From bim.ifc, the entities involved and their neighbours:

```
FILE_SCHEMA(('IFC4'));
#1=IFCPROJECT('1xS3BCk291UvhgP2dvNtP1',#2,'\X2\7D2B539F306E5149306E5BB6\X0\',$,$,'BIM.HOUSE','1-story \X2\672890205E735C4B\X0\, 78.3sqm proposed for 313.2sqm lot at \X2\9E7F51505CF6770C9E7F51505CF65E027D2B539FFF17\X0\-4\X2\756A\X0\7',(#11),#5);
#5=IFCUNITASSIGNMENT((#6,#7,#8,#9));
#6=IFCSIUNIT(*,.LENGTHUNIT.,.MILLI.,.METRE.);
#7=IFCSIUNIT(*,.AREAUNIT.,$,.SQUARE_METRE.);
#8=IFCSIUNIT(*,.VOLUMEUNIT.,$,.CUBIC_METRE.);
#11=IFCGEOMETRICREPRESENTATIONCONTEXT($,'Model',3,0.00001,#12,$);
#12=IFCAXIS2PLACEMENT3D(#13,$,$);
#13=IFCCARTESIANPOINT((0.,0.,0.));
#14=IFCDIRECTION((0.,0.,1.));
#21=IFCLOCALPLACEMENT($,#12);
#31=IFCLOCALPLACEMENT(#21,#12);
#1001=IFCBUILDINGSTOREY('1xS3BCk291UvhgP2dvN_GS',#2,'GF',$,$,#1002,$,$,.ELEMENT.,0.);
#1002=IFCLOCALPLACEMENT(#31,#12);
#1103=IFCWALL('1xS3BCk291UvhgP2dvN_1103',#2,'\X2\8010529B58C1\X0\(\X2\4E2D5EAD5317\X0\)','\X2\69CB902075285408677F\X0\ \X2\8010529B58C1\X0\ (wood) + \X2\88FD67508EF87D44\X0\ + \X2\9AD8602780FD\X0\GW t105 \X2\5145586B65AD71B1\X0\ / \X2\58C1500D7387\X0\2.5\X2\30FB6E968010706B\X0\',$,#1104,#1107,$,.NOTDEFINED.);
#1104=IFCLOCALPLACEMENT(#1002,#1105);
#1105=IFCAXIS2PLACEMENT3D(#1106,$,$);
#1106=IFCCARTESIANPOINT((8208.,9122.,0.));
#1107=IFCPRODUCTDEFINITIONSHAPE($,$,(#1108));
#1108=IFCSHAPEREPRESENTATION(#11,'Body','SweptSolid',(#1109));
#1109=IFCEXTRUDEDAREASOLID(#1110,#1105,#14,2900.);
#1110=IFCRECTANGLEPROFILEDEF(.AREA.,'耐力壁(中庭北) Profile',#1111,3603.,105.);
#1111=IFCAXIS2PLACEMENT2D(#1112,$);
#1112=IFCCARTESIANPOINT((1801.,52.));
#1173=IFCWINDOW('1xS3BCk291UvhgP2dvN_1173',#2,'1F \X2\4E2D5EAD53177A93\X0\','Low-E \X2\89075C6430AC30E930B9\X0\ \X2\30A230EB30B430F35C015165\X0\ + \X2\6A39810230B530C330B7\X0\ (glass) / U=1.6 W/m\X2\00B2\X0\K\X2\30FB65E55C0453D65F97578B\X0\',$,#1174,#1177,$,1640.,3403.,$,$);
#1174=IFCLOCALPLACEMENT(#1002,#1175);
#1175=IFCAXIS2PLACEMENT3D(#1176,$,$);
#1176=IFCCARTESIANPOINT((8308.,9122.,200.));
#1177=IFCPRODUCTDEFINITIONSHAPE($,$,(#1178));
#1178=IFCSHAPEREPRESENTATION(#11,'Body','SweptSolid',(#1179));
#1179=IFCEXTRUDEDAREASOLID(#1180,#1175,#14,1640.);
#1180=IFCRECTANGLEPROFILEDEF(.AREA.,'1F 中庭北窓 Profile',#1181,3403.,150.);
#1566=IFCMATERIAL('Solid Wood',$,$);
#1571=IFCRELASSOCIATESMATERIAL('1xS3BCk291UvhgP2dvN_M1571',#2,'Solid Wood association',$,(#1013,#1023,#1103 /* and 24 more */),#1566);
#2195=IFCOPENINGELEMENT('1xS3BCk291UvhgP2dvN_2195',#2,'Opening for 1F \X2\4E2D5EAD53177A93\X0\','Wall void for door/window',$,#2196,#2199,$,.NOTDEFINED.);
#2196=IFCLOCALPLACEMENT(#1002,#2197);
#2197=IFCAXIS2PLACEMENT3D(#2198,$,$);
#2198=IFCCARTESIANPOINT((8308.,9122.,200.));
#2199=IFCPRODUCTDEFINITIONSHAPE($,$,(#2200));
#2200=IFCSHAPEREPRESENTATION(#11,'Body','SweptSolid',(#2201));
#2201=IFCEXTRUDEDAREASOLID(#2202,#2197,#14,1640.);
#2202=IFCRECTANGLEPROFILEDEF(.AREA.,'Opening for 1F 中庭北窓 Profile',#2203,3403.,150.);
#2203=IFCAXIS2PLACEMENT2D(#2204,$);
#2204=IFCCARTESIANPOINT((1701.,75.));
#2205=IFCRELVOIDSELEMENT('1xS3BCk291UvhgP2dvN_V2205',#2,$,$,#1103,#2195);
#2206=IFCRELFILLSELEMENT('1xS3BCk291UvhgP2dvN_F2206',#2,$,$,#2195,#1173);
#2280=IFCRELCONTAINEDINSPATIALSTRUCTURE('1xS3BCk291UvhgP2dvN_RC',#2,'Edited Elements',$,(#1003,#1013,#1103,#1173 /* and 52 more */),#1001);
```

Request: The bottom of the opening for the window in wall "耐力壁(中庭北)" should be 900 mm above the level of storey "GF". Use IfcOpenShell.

```python
import numpy as np
import ifcopenshell
import ifcopenshell.api.geometry
import ifcopenshell.geom
import ifcopenshell.util.element
import ifcopenshell.util.placement
import ifcopenshell.util.shape
import ifcopenshell.util.unit

model = ifcopenshell.open("bim.ifc")
unit_scale = ifcopenshell.util.unit.calculate_unit_scale(model)

window = model.by_id(1173)
opening = window.FillsVoids[0].RelatingOpeningElement
storey = ifcopenshell.util.element.get_container(window, ifc_class="IfcBuildingStorey")
level = ifcopenshell.util.placement.get_local_placement(storey.ObjectPlacement)[2, 3]

# The opening's origin need not be at the sill, so measure its lowest point.
shape = ifcopenshell.geom.create_shape(ifcopenshell.geom.settings(), opening)
bottom = ifcopenshell.util.shape.get_shape_bottom_elevation(shape, shape.geometry) / unit_scale
dz = level + 0.9 / unit_scale - bottom

shift = np.array([0.0, 0.0, dz])
# The window is not placed relative to its opening, so move both.
for product in (opening, window):
    matrix = ifcopenshell.util.placement.get_local_placement(product.ObjectPlacement)
    matrix[:3, 3] += shift
    ifcopenshell.api.geometry.edit_object_placement(model, product=product, matrix=matrix, is_si=False)

print(f"moved by {dz * unit_scale:+.3f} m")

model.write("bim_updated.ifc")
```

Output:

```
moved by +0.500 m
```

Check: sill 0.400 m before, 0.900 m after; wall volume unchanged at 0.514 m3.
